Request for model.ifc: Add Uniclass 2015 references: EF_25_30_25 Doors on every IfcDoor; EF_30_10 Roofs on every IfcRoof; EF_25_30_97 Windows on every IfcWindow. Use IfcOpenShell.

First a look at what the model holds.

```python
import ifcopenshell

model = ifcopenshell.open("model.ifc")
print(model.schema)
print("classifications:", [c.Name for c in model.by_type("IfcClassification")])
for ifc_class in ("IfcDoor", "IfcRoof", "IfcStair", "IfcWall", "IfcWindow"):
    print(ifc_class, len(model.by_type(ifc_class)))
```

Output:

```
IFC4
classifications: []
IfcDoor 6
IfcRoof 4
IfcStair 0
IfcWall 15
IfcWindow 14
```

```python
import ifcopenshell
import ifcopenshell.api.classification

model = ifcopenshell.open("model.ifc")

system = ifcopenshell.api.classification.add_classification(model, classification="Uniclass 2015")

codes = {
    "IfcDoor": ("EF_25_30_25", "Doors"),
    "IfcRoof": ("EF_30_10", "Roofs"),
    "IfcWindow": ("EF_25_30_97", "Windows"),
}
for ifc_class, (code, name) in codes.items():
    products = model.by_type(ifc_class)
    ifcopenshell.api.classification.add_reference(
        model, products=products, classification=system, identification=code, name=name
    )
    print(code, len(products))

model.write("model_updated.ifc")
```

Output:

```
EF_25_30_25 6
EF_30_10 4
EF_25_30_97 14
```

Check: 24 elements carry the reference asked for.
